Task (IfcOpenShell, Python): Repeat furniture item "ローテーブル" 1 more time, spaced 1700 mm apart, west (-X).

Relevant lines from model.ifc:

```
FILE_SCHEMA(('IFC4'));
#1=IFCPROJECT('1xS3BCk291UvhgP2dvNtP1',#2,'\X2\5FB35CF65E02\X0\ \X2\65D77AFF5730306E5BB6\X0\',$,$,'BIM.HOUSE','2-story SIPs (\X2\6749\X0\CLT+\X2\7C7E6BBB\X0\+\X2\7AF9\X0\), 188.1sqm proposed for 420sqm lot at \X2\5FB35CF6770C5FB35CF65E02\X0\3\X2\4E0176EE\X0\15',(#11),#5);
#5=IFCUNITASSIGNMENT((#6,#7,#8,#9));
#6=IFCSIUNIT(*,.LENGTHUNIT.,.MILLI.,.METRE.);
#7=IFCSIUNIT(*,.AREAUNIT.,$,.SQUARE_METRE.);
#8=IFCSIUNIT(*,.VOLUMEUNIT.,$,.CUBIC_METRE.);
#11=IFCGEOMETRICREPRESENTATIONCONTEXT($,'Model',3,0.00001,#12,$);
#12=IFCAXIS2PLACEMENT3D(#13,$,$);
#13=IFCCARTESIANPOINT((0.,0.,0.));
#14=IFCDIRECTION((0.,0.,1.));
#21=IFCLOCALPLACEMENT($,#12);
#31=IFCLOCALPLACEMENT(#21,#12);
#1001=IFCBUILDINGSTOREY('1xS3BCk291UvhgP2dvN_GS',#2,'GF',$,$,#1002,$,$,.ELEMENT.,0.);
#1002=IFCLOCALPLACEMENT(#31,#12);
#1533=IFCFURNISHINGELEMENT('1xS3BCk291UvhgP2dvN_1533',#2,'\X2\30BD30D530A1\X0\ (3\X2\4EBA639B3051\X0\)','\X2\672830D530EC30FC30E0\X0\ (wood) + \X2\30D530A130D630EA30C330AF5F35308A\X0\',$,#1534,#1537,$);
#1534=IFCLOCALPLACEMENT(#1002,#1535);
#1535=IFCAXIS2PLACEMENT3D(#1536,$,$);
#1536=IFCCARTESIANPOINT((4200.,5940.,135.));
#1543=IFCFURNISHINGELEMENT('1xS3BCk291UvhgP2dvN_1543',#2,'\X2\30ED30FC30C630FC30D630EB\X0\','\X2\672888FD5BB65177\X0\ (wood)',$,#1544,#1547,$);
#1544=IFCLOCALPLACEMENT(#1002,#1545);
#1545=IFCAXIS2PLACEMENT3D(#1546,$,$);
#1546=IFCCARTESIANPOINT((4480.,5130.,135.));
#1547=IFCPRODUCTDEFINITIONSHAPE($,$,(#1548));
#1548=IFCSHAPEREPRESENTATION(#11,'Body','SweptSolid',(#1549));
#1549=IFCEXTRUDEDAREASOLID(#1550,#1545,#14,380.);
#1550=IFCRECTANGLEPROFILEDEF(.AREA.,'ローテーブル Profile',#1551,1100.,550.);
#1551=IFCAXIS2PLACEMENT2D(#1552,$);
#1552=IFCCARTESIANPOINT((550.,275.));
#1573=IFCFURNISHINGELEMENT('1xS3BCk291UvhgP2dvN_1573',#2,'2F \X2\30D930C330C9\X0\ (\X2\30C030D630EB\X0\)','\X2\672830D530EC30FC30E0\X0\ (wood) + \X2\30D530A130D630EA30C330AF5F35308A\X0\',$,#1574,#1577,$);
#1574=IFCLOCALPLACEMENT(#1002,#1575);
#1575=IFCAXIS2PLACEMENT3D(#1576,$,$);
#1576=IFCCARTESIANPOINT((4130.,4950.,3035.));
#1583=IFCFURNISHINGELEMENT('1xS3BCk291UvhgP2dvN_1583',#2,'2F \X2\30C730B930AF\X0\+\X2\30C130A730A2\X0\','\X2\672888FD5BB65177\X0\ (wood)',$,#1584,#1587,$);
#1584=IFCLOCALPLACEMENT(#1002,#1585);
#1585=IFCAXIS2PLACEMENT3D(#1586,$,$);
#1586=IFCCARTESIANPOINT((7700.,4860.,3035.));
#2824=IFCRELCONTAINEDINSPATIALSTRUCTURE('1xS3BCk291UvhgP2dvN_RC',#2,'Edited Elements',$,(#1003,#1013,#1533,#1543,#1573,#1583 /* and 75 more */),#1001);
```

```python
import numpy as np
import ifcopenshell
import ifcopenshell.api.geometry
import ifcopenshell.api.root
import ifcopenshell.util.element
import ifcopenshell.util.placement
import ifcopenshell.util.unit

model = ifcopenshell.open("model.ifc")
unit_scale = ifcopenshell.util.unit.calculate_unit_scale(model)


def reuse_history(source, copy):
    """copy_class also copies each property set's owner history, people and application; keep the originals."""
    for rel in copy.IsDefinedBy:
        if rel.is_a("IfcRelDefinesByProperties") and (history := rel.RelatingPropertyDefinition.OwnerHistory):
            rel.RelatingPropertyDefinition.OwnerHistory = source.OwnerHistory
            ifcopenshell.util.element.remove_deep2(model, history)


source = model.by_id(1543)
base = ifcopenshell.util.placement.get_local_placement(source.ObjectPlacement)
step = np.array([-1.0, 0.0, 0.0]) * 1.7 / unit_scale

for i in range(1, 2):
    copy = ifcopenshell.api.root.copy_class(model, product=source)
    copy.Representation = ifcopenshell.util.element.copy_deep(
        model, source.Representation, exclude=["IfcGeometricRepresentationContext", "IfcRepresentationMap"]
    )
    reuse_history(source, copy)
    matrix = base.copy()
    matrix[:3, 3] += i * step
    print("added at", matrix[:3, 3].round(3) + 0.0)
    ifcopenshell.api.geometry.edit_object_placement(model, product=copy, matrix=matrix, is_si=False)

model.write("model_v2.ifc")
```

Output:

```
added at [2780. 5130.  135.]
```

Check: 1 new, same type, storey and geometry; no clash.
